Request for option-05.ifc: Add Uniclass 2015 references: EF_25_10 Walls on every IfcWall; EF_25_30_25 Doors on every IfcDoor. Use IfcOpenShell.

First a look at what the model holds.

```python
import ifcopenshell

model = ifcopenshell.open("option-05.ifc")
print(model.schema)
print("classifications:", [c.Name for c in model.by_type("IfcClassification")])
for ifc_class in ("IfcDoor", "IfcRoof", "IfcStair", "IfcWall", "IfcWindow"):
    print(ifc_class, len(model.by_type(ifc_class)))
```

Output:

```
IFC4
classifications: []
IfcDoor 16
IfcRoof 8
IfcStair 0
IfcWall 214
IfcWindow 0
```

```python
import ifcopenshell
import ifcopenshell.api.classification

model = ifcopenshell.open("option-05.ifc")

system = ifcopenshell.api.classification.add_classification(model, classification="Uniclass 2015")

codes = {
    "IfcWall": ("EF_25_10", "Walls"),
    "IfcDoor": ("EF_25_30_25", "Doors"),
}
for ifc_class, (code, name) in codes.items():
    products = model.by_type(ifc_class)
    ifcopenshell.api.classification.add_reference(
        model, products=products, classification=system, identification=code, name=name
    )
    print(code, len(products))

model.write("option-05_v2.ifc")
```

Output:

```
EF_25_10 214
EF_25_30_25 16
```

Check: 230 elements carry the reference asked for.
